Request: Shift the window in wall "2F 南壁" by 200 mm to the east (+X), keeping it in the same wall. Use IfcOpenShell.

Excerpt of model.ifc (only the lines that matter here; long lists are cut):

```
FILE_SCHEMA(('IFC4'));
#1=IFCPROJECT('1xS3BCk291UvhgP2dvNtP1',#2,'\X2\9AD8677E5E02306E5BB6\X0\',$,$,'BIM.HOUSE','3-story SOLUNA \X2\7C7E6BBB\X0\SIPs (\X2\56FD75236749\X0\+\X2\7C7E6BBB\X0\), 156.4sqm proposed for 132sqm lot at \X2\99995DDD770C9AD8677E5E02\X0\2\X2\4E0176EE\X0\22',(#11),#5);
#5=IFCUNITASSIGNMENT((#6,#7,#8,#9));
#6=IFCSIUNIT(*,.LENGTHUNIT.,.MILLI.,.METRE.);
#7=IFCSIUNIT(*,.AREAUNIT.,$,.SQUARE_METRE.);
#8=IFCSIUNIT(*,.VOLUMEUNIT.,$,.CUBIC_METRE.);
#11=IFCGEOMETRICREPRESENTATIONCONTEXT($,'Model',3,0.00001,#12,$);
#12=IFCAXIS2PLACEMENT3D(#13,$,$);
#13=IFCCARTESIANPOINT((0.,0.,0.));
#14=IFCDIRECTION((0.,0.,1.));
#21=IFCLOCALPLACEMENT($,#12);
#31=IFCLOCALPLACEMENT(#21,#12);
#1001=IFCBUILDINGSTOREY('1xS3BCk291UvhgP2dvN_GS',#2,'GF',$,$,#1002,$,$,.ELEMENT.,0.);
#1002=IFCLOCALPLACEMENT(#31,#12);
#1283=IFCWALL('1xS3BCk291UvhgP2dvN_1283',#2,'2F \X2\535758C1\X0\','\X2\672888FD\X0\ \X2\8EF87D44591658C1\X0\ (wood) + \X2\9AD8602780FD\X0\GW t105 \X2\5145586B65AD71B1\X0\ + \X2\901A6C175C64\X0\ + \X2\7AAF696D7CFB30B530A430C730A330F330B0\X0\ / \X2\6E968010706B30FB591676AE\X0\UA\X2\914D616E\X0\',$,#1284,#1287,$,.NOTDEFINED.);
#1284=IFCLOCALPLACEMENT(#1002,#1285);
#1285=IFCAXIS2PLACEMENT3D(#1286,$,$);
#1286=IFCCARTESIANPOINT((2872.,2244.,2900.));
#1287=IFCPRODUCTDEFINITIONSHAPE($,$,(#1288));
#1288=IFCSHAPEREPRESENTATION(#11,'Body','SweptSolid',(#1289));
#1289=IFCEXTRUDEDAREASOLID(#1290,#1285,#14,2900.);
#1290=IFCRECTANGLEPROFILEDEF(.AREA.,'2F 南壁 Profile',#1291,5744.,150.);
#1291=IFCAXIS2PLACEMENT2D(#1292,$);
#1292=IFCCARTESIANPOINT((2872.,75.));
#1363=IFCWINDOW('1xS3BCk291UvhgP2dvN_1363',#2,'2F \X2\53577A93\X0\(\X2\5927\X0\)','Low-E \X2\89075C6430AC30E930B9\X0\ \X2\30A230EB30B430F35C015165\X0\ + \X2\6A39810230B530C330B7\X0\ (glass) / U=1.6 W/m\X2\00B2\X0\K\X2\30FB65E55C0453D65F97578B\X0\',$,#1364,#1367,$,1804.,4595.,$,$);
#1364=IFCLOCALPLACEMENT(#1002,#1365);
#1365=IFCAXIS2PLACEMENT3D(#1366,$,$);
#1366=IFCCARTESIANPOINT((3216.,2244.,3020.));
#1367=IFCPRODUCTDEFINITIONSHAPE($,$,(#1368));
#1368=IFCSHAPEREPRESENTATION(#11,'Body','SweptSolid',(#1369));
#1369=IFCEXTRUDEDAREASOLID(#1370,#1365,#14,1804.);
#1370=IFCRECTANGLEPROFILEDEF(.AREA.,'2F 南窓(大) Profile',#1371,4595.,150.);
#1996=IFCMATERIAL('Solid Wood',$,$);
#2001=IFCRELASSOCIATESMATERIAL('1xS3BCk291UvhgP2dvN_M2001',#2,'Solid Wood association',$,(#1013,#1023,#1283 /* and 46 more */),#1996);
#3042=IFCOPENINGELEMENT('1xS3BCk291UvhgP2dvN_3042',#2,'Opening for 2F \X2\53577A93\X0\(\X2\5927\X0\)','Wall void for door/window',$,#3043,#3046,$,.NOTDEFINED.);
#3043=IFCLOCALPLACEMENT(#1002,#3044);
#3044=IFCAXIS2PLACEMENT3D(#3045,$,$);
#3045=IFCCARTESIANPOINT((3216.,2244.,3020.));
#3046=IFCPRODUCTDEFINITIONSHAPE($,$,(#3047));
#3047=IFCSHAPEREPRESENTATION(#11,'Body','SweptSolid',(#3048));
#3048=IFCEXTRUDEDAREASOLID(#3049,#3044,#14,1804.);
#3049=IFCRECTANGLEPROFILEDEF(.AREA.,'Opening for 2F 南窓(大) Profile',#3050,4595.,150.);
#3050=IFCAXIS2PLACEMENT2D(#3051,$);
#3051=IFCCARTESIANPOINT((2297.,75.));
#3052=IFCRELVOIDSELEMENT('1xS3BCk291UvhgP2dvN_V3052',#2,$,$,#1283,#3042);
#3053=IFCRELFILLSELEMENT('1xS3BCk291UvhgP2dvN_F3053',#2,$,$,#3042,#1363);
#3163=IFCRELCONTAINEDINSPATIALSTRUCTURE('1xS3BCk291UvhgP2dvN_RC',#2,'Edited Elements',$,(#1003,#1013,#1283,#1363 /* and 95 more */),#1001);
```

```python
import ifcopenshell
import ifcopenshell.api.geometry
import ifcopenshell.util.placement
import ifcopenshell.util.unit

model = ifcopenshell.open("model.ifc")
unit_scale = ifcopenshell.util.unit.calculate_unit_scale(model)

window = model.by_guid("1xS3BCk291UvhgP2dvN_1363")
opening = window.FillsVoids[0].RelatingOpeningElement
wall = opening.VoidsElements[0].RelatingBuildingElement

wall_matrix = ifcopenshell.util.placement.get_local_placement(wall.ObjectPlacement)
shift = wall_matrix[:3, 0] * 0.2 / unit_scale
before = ifcopenshell.util.placement.get_local_placement(window.ObjectPlacement)[:3, 3].copy()

# The window is not placed relative to its opening, so move both.
for product in (opening, window):
    matrix = ifcopenshell.util.placement.get_local_placement(product.ObjectPlacement)
    matrix[:3, 3] += shift
    ifcopenshell.api.geometry.edit_object_placement(model, product=product, matrix=matrix, is_si=False)

after = ifcopenshell.util.placement.get_local_placement(window.ObjectPlacement)[:3, 3]
print("window moved by", (after - before).round(3) + 0.0)

model.write("model-out.ifc")
```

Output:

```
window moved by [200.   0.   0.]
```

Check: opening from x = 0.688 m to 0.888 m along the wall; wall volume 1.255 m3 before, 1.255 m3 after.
